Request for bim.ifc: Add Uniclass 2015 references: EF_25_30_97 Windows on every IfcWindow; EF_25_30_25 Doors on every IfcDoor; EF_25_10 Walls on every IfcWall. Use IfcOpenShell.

First a look at what the model holds.

```python
import ifcopenshell

model = ifcopenshell.open("bim.ifc")
print(model.schema)
print("classifications:", [c.Name for c in model.by_type("IfcClassification")])
for ifc_class in ("IfcDoor", "IfcRoof", "IfcStair", "IfcWall", "IfcWindow"):
    print(ifc_class, len(model.by_type(ifc_class)))
```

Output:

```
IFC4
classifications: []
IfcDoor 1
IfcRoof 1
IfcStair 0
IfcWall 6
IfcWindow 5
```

```python
import ifcopenshell
import ifcopenshell.api.classification

model = ifcopenshell.open("bim.ifc")

system = ifcopenshell.api.classification.add_classification(model, classification="Uniclass 2015")

codes = {
    "IfcWindow": ("EF_25_30_97", "Windows"),
    "IfcDoor": ("EF_25_30_25", "Doors"),
    "IfcWall": ("EF_25_10", "Walls"),
}
for ifc_class, (code, name) in codes.items():
    products = model.by_type(ifc_class)
    ifcopenshell.api.classification.add_reference(
        model, products=products, classification=system, identification=code, name=name
    )
    print(code, len(products))

model.write("bim_updated.ifc")
```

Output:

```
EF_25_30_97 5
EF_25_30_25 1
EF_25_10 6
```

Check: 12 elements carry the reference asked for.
